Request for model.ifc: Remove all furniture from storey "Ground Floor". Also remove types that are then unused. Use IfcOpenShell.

First a look at what the model holds.

```python
import ifcopenshell
import ifcopenshell.util.element

model = ifcopenshell.open("model.ifc")
print(model.schema)
storey = next(s for s in model.by_type("IfcBuildingStorey") if s.Name == "Ground Floor")
furniture = [e for e in ifcopenshell.util.element.get_decomposition(storey) if e.is_a("IfcFurnishingElement")]
seen = {}
for e in furniture:
    element_type = ifcopenshell.util.element.get_type(e)
    name = element_type.Name if element_type not in (None, e) else None
    seen[name] = seen.get(name, 0) + 1
for name, count in sorted(seen.items(), key=str):
    print(count, "x", name)
```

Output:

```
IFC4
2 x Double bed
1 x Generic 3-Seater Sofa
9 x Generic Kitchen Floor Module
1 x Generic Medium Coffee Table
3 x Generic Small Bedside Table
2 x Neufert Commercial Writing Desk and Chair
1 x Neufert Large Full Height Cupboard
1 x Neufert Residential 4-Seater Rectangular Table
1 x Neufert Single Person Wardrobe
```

```python
import ifcopenshell
import ifcopenshell.api.root
import ifcopenshell.util.element

model = ifcopenshell.open("model.ifc")

storey = next(s for s in model.by_type("IfcBuildingStorey") if s.Name == "Ground Floor")
furniture = [e for e in ifcopenshell.util.element.get_decomposition(storey) if e.is_a("IfcFurnishingElement")]
types = {ifcopenshell.util.element.get_type(e) for e in furniture} - {None, *furniture}

for e in furniture:
    ifcopenshell.api.root.remove_product(model, product=e)
print(len(furniture), "removed")

unused = [t for t in types if not ifcopenshell.util.element.get_types(t)]
for t in unused:
    ifcopenshell.api.root.remove_product(model, product=t)
print(len(unused), "unused types removed")

model.write("model-out.ifc")
```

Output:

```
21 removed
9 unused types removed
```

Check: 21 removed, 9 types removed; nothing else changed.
